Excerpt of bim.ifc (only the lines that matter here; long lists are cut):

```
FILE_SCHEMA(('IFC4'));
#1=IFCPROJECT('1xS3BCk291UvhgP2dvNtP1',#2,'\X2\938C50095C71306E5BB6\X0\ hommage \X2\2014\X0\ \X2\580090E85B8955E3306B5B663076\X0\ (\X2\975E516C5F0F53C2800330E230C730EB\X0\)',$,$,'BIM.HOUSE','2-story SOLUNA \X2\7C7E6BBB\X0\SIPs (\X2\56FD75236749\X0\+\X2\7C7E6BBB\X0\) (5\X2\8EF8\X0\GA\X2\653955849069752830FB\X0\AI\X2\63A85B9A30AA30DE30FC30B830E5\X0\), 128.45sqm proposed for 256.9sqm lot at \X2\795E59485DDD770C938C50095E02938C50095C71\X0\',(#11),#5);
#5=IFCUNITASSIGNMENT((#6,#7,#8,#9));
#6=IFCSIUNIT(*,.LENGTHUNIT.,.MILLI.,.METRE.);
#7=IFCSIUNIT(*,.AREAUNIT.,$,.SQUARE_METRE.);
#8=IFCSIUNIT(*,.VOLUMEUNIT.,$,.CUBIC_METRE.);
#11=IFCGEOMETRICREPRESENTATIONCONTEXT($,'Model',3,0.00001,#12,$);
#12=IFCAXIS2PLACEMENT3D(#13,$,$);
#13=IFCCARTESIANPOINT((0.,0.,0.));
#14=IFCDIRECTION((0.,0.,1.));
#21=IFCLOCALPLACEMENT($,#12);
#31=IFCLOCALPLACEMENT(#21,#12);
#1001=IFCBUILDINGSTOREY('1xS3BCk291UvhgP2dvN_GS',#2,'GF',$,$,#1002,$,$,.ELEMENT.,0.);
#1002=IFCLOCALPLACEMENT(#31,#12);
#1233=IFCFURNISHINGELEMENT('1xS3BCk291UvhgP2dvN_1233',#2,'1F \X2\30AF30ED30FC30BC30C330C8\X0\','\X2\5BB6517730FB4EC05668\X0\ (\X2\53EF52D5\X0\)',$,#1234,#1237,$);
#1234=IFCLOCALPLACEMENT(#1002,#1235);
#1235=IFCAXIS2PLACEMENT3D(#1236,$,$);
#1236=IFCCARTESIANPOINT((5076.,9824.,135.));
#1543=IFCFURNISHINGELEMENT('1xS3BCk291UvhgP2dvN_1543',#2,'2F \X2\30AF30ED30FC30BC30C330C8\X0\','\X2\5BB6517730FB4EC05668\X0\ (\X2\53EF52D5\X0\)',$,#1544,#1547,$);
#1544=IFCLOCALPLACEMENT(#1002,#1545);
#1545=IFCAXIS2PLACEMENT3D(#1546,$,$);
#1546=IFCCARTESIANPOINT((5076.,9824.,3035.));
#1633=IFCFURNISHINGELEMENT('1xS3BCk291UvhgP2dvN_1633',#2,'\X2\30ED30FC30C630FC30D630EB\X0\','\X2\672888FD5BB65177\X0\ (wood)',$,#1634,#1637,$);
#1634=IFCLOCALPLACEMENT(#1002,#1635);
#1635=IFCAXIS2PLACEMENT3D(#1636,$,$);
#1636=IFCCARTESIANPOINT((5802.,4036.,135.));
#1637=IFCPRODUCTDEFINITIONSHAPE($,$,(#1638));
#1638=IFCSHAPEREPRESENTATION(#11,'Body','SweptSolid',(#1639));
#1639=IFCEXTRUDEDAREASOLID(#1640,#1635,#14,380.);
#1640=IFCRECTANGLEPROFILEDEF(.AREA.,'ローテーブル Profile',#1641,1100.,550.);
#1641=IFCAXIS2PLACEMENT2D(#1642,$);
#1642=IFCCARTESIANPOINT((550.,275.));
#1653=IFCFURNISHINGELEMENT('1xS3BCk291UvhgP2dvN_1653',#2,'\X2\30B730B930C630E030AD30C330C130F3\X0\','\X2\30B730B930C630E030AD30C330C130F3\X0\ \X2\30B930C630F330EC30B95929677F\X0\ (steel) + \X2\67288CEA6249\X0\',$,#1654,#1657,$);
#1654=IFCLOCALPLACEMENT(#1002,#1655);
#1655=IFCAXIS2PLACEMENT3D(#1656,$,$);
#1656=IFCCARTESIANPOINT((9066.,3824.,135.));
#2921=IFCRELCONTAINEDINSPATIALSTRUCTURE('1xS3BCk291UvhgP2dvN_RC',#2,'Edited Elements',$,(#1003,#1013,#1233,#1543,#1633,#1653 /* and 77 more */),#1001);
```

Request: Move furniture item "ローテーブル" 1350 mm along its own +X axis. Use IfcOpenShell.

```python
import ifcopenshell
import ifcopenshell.api.geometry
import ifcopenshell.util.placement
import ifcopenshell.util.unit

model = ifcopenshell.open("bim.ifc")
unit_scale = ifcopenshell.util.unit.calculate_unit_scale(model)

item = model.by_id(1633)
matrix = ifcopenshell.util.placement.get_local_placement(item.ObjectPlacement)
matrix[:3, 3] += matrix[:3, 0] * 1.35 / unit_scale
ifcopenshell.api.geometry.edit_object_placement(model, product=item, matrix=matrix, is_si=False)

print(ifcopenshell.util.placement.get_local_placement(item.ObjectPlacement).round(3) + 0.0)

model.write("bim_v2.ifc")
```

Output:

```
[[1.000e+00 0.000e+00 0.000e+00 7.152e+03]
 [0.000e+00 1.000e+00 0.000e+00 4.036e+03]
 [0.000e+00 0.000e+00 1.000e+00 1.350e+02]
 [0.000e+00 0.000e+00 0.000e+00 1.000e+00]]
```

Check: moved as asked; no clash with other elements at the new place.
